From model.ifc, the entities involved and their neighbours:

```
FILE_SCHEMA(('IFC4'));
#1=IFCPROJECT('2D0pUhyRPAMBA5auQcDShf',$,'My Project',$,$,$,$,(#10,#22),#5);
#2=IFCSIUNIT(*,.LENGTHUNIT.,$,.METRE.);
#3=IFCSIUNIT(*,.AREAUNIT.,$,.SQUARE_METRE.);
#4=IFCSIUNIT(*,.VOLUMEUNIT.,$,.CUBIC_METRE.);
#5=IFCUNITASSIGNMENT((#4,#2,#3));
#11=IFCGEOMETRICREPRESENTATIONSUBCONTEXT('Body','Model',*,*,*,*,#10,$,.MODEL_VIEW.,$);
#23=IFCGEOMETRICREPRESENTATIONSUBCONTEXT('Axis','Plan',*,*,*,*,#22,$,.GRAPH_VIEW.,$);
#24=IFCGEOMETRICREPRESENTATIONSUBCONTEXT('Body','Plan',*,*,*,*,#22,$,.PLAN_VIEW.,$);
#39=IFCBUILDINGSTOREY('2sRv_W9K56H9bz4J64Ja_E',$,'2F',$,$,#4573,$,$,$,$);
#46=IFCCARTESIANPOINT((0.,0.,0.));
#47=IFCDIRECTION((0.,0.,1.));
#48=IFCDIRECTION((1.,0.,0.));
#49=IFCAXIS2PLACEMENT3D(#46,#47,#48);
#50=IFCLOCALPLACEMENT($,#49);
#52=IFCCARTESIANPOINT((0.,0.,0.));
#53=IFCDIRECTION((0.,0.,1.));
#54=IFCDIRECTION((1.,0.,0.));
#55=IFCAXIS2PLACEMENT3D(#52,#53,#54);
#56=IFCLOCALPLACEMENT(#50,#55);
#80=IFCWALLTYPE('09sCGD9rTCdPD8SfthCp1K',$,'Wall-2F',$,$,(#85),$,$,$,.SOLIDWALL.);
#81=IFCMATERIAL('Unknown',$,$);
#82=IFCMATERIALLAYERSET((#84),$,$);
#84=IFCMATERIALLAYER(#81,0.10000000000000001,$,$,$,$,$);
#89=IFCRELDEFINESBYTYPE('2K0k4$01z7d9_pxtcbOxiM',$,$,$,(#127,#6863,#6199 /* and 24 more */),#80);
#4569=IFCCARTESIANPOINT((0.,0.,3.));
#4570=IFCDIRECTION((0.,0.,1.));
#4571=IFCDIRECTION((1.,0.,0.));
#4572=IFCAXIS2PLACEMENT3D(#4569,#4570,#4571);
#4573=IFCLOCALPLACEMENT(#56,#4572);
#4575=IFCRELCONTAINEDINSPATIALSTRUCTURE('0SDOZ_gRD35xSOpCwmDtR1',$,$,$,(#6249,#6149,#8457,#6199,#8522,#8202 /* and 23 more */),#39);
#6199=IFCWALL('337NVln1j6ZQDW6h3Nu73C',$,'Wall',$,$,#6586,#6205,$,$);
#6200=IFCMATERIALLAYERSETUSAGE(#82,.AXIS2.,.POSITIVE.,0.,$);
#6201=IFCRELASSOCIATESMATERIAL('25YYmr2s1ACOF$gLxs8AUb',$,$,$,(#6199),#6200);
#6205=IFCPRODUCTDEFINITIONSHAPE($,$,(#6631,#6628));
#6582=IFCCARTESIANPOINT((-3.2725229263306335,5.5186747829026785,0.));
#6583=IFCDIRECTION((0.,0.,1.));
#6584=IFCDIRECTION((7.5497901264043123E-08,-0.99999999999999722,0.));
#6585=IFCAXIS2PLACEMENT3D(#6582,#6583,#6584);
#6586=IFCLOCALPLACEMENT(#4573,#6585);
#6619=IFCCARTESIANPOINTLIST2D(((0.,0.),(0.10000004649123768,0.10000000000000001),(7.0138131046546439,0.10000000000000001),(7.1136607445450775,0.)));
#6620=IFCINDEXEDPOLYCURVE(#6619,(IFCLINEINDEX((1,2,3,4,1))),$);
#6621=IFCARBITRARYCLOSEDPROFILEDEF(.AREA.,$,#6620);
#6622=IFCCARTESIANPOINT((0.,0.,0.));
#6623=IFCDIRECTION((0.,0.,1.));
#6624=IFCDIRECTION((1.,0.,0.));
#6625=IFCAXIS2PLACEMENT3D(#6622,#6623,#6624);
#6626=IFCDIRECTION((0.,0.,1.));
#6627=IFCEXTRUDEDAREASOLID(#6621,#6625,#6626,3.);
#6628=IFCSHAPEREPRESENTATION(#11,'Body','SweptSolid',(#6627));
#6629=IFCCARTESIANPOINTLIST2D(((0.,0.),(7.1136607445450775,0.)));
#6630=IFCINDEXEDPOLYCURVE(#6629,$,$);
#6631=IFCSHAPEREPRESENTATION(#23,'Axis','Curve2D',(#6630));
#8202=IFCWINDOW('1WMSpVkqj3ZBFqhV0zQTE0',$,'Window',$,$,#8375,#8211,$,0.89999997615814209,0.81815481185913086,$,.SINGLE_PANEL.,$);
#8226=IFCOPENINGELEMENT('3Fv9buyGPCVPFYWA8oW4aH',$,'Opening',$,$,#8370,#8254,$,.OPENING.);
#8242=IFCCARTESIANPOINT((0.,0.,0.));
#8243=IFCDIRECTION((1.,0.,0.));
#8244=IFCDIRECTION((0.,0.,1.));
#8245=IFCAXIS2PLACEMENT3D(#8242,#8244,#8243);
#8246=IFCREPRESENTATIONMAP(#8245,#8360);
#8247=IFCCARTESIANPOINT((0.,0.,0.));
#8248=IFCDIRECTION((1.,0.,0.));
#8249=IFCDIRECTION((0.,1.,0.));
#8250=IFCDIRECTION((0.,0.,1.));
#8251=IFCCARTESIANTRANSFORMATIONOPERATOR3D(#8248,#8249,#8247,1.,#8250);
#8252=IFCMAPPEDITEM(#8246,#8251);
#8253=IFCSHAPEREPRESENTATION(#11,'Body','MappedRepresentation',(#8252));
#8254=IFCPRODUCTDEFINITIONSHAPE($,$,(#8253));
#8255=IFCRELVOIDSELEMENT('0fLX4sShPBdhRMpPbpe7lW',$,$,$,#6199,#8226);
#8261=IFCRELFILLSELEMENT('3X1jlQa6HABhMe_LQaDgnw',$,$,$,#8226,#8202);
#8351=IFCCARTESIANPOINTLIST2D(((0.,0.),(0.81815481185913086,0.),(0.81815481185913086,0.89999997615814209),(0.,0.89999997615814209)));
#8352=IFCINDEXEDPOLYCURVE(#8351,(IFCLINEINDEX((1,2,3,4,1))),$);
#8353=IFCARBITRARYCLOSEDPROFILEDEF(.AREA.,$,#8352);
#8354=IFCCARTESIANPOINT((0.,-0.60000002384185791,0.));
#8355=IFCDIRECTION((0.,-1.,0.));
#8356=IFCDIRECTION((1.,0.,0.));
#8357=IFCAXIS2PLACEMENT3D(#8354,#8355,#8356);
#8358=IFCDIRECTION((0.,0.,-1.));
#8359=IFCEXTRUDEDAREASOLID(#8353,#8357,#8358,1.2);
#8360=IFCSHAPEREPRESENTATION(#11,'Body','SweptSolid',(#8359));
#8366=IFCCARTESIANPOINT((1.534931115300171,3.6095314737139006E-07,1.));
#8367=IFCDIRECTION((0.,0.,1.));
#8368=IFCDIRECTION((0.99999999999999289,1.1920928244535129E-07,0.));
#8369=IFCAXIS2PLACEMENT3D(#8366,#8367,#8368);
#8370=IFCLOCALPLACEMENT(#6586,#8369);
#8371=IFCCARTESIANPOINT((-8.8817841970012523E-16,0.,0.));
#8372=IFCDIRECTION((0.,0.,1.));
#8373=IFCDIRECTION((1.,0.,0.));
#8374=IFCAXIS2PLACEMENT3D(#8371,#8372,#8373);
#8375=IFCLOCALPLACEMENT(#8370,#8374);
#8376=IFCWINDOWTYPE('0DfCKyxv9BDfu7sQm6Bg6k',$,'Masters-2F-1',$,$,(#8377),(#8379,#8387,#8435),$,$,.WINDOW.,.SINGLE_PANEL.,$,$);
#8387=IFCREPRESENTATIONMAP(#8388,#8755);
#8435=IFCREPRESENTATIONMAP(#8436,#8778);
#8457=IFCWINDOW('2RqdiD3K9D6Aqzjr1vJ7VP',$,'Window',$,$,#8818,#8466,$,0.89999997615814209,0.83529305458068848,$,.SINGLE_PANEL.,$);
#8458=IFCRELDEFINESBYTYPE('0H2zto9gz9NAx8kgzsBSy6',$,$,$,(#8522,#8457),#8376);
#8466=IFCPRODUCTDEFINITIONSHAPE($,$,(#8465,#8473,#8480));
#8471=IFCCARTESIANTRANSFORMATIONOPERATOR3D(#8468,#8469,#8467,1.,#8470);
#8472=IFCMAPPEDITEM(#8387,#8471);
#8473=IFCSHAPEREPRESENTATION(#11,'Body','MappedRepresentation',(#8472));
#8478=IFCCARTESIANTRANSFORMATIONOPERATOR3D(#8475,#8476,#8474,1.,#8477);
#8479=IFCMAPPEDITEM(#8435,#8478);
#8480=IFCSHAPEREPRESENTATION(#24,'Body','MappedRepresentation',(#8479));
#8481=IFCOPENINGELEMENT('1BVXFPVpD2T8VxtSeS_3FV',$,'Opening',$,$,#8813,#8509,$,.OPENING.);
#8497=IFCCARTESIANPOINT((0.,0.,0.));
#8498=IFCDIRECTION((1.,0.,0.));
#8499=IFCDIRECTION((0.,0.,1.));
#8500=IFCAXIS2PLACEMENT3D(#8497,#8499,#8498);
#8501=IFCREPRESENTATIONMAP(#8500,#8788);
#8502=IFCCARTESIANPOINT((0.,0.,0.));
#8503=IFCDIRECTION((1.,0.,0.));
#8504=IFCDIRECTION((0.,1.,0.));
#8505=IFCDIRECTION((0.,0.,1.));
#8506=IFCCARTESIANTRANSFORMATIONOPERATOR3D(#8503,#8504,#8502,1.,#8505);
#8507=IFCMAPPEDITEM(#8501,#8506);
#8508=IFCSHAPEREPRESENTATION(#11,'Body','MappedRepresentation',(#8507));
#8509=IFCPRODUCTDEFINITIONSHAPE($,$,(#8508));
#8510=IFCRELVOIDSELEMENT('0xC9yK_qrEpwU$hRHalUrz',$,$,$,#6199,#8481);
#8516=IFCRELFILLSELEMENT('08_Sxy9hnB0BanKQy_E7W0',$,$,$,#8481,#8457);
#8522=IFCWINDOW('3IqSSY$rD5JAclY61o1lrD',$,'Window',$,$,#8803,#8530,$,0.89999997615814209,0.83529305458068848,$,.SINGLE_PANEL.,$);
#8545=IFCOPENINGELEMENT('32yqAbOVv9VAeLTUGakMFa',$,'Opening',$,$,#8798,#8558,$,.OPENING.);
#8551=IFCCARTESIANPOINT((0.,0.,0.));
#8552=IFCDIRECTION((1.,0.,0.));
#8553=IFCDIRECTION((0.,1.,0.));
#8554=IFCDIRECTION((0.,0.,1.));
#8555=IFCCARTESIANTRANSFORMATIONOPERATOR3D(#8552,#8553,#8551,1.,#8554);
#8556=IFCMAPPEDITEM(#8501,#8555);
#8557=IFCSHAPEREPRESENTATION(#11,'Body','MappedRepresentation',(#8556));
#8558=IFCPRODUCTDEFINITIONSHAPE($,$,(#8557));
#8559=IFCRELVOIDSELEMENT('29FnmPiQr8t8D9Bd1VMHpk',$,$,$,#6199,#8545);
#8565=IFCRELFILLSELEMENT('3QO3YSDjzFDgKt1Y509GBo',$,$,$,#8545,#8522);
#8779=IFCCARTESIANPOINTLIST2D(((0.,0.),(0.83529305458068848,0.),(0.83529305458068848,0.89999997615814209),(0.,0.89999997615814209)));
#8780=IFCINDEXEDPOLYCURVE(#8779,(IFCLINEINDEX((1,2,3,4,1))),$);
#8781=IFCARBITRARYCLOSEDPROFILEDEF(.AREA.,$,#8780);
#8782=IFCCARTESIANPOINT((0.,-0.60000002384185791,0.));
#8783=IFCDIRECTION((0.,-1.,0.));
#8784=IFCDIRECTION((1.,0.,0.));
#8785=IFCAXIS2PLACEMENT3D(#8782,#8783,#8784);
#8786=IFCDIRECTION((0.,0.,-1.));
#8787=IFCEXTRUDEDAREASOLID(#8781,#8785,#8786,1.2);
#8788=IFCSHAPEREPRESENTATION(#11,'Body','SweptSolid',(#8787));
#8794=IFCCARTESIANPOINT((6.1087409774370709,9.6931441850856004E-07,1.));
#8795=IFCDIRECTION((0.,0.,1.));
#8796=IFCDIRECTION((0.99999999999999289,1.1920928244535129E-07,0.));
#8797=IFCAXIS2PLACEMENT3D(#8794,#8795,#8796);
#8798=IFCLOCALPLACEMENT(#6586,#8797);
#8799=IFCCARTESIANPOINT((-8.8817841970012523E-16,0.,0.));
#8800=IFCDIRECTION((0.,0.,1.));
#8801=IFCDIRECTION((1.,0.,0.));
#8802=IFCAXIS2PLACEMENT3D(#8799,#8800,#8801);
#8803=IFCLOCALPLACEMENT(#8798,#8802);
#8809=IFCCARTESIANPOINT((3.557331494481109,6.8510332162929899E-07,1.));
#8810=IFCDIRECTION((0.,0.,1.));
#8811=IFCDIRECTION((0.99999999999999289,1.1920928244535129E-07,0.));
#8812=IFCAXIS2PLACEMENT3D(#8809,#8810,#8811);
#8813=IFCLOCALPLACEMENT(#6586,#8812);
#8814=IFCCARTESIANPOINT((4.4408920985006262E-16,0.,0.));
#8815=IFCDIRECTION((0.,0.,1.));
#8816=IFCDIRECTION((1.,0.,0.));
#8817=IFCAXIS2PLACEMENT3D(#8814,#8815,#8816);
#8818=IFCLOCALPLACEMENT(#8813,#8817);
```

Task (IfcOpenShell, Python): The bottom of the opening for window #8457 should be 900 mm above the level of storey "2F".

```python
import numpy as np
import ifcopenshell
import ifcopenshell.api.geometry
import ifcopenshell.geom
import ifcopenshell.util.element
import ifcopenshell.util.placement
import ifcopenshell.util.shape
import ifcopenshell.util.unit

model = ifcopenshell.open("model.ifc")
unit_scale = ifcopenshell.util.unit.calculate_unit_scale(model)

window = model.by_guid("2RqdiD3K9D6Aqzjr1vJ7VP")
opening = window.FillsVoids[0].RelatingOpeningElement
storey = ifcopenshell.util.element.get_container(window, ifc_class="IfcBuildingStorey")
level = ifcopenshell.util.placement.get_local_placement(storey.ObjectPlacement)[2, 3]

# The opening's origin need not be at the sill, so measure its lowest point.
shape = ifcopenshell.geom.create_shape(ifcopenshell.geom.settings(), opening)
bottom = ifcopenshell.util.shape.get_shape_bottom_elevation(shape, shape.geometry) / unit_scale
dz = level + 0.9 - bottom

shift = np.array([0.0, 0.0, dz])
# The window is placed relative to its opening, so it follows when the opening moves.
matrix = ifcopenshell.util.placement.get_local_placement(opening.ObjectPlacement)
matrix[:3, 3] += shift
ifcopenshell.api.geometry.edit_object_placement(
    model, product=opening, matrix=matrix, is_si=False, should_transform_children=True
)

print(f"moved by {dz * unit_scale:+.3f} m")

model.write("model-out.ifc")
```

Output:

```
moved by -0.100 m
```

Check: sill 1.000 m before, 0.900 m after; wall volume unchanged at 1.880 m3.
